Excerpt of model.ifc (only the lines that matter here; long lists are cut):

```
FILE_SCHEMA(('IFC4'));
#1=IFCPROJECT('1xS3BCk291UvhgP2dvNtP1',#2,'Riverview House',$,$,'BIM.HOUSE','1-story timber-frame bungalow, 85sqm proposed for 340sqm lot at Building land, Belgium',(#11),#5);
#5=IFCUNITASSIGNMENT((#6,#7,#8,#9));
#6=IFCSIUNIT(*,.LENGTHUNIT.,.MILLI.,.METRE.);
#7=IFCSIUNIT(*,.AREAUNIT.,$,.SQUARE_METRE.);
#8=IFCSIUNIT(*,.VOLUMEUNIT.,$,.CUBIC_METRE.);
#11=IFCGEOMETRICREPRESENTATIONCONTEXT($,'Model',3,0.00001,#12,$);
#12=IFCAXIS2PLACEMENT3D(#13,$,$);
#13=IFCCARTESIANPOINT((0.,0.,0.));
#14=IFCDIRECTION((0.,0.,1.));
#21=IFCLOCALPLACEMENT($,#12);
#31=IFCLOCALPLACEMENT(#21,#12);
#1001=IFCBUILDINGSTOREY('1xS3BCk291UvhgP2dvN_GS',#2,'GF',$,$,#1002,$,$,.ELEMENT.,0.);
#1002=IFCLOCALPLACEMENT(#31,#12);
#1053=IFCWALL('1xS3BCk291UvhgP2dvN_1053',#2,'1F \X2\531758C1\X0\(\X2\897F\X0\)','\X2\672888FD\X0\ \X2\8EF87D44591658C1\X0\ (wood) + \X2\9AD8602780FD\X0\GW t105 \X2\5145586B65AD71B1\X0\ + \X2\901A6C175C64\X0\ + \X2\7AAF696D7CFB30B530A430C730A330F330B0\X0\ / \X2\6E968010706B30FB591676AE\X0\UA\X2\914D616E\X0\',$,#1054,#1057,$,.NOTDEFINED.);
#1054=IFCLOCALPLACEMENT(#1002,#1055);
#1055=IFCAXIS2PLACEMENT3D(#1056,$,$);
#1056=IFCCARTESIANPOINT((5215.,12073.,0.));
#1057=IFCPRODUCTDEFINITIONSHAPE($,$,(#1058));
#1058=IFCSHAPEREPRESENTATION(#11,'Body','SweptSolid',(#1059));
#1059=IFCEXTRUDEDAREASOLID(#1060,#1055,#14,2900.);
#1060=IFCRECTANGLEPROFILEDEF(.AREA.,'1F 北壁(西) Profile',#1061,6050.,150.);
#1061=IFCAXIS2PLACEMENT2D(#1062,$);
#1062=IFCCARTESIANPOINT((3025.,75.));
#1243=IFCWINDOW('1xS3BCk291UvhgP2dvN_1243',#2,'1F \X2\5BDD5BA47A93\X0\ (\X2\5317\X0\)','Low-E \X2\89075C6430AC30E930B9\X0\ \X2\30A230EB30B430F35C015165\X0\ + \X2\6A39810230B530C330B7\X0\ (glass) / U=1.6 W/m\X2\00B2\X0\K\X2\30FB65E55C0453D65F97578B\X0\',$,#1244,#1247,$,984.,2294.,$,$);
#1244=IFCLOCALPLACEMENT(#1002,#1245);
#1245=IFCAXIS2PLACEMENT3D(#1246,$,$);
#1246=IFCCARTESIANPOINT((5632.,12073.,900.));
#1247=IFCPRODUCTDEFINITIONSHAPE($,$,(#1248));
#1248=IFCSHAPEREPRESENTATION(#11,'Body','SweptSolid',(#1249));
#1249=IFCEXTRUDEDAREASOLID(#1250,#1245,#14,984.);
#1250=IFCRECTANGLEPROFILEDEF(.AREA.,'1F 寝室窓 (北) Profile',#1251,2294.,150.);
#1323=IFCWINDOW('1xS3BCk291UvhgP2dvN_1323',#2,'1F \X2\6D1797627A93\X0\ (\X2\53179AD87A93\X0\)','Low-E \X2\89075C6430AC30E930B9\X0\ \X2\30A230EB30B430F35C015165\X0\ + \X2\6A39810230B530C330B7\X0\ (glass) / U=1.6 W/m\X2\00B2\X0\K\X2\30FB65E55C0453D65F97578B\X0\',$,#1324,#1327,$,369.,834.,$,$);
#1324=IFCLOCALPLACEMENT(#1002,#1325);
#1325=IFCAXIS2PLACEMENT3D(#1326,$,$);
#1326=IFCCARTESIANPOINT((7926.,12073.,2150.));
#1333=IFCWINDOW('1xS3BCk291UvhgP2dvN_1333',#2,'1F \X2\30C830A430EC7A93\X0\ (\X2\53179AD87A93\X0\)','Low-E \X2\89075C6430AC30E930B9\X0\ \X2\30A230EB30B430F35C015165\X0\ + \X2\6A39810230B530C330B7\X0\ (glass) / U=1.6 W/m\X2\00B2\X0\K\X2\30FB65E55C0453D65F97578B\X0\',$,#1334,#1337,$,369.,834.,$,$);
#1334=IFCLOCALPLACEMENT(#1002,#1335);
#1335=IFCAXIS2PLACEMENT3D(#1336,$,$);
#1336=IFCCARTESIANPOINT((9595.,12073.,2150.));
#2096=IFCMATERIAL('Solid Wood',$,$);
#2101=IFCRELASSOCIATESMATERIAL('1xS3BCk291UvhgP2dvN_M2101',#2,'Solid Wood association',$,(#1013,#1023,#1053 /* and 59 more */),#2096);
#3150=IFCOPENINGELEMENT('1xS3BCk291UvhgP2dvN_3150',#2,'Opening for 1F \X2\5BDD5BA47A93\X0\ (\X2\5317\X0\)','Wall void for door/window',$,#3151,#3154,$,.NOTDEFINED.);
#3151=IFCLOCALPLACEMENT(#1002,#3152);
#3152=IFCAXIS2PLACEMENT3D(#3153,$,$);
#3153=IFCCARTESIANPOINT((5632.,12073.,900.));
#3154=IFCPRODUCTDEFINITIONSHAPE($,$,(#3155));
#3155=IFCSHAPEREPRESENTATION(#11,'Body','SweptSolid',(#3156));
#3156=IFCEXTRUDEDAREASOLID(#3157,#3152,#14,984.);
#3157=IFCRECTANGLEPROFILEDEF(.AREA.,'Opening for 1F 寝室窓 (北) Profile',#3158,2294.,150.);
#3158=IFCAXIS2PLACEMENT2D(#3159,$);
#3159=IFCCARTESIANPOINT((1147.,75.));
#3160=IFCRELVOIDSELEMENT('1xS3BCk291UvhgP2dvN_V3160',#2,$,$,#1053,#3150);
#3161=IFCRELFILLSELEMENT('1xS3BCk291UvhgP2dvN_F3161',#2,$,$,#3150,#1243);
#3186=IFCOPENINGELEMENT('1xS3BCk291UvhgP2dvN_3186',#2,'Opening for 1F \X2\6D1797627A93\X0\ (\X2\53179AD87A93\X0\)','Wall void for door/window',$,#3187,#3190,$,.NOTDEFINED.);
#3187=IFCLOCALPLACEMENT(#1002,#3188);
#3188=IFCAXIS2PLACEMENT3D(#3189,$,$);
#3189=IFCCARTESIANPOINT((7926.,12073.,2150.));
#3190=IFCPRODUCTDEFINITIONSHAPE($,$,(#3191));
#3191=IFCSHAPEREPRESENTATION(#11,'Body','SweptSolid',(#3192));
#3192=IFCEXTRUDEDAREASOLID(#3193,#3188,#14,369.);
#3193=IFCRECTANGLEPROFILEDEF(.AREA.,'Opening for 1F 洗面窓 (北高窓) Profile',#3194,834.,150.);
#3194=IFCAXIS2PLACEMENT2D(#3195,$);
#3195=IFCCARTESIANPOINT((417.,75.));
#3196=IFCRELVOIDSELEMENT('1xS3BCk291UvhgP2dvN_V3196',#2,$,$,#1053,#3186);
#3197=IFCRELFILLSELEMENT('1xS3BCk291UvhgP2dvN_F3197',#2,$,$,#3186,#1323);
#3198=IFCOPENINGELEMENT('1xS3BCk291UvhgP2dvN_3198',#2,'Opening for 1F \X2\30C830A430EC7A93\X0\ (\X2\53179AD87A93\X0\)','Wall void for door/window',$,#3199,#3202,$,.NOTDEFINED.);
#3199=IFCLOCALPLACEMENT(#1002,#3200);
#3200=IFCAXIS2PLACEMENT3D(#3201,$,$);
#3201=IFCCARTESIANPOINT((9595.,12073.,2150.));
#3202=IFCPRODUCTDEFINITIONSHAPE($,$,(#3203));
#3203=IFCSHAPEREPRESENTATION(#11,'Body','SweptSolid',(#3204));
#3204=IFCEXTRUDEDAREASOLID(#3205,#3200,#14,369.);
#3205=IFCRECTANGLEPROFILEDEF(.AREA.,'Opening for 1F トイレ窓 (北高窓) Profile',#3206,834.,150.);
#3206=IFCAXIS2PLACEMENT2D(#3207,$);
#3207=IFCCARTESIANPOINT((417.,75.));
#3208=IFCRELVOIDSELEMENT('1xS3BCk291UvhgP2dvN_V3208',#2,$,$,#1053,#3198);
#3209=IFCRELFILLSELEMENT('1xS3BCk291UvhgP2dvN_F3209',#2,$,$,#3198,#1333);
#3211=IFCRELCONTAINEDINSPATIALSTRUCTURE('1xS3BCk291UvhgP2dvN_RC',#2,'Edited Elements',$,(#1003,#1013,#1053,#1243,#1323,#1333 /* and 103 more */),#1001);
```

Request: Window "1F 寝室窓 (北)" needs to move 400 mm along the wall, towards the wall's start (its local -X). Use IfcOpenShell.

```python
import ifcopenshell
import ifcopenshell.api.geometry
import ifcopenshell.util.placement

model = ifcopenshell.open("model.ifc")

window = model.by_guid("1xS3BCk291UvhgP2dvN_1243")
opening = window.FillsVoids[0].RelatingOpeningElement
wall = opening.VoidsElements[0].RelatingBuildingElement

wall_matrix = ifcopenshell.util.placement.get_local_placement(wall.ObjectPlacement)
shift = wall_matrix[:3, 0] * -400.0
before = ifcopenshell.util.placement.get_local_placement(window.ObjectPlacement)[:3, 3].copy()

# The window is not placed relative to its opening, so move both.
for product in (opening, window):
    matrix = ifcopenshell.util.placement.get_local_placement(product.ObjectPlacement)
    matrix[:3, 3] += shift
    ifcopenshell.api.geometry.edit_object_placement(model, product=product, matrix=matrix, is_si=False)

after = ifcopenshell.util.placement.get_local_placement(window.ObjectPlacement)[:3, 3]
print("window moved by", (after - before).round(3) + 0.0)

model.write("model_edited.ifc")
```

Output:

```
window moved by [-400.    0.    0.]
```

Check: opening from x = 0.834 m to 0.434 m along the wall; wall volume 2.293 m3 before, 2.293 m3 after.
